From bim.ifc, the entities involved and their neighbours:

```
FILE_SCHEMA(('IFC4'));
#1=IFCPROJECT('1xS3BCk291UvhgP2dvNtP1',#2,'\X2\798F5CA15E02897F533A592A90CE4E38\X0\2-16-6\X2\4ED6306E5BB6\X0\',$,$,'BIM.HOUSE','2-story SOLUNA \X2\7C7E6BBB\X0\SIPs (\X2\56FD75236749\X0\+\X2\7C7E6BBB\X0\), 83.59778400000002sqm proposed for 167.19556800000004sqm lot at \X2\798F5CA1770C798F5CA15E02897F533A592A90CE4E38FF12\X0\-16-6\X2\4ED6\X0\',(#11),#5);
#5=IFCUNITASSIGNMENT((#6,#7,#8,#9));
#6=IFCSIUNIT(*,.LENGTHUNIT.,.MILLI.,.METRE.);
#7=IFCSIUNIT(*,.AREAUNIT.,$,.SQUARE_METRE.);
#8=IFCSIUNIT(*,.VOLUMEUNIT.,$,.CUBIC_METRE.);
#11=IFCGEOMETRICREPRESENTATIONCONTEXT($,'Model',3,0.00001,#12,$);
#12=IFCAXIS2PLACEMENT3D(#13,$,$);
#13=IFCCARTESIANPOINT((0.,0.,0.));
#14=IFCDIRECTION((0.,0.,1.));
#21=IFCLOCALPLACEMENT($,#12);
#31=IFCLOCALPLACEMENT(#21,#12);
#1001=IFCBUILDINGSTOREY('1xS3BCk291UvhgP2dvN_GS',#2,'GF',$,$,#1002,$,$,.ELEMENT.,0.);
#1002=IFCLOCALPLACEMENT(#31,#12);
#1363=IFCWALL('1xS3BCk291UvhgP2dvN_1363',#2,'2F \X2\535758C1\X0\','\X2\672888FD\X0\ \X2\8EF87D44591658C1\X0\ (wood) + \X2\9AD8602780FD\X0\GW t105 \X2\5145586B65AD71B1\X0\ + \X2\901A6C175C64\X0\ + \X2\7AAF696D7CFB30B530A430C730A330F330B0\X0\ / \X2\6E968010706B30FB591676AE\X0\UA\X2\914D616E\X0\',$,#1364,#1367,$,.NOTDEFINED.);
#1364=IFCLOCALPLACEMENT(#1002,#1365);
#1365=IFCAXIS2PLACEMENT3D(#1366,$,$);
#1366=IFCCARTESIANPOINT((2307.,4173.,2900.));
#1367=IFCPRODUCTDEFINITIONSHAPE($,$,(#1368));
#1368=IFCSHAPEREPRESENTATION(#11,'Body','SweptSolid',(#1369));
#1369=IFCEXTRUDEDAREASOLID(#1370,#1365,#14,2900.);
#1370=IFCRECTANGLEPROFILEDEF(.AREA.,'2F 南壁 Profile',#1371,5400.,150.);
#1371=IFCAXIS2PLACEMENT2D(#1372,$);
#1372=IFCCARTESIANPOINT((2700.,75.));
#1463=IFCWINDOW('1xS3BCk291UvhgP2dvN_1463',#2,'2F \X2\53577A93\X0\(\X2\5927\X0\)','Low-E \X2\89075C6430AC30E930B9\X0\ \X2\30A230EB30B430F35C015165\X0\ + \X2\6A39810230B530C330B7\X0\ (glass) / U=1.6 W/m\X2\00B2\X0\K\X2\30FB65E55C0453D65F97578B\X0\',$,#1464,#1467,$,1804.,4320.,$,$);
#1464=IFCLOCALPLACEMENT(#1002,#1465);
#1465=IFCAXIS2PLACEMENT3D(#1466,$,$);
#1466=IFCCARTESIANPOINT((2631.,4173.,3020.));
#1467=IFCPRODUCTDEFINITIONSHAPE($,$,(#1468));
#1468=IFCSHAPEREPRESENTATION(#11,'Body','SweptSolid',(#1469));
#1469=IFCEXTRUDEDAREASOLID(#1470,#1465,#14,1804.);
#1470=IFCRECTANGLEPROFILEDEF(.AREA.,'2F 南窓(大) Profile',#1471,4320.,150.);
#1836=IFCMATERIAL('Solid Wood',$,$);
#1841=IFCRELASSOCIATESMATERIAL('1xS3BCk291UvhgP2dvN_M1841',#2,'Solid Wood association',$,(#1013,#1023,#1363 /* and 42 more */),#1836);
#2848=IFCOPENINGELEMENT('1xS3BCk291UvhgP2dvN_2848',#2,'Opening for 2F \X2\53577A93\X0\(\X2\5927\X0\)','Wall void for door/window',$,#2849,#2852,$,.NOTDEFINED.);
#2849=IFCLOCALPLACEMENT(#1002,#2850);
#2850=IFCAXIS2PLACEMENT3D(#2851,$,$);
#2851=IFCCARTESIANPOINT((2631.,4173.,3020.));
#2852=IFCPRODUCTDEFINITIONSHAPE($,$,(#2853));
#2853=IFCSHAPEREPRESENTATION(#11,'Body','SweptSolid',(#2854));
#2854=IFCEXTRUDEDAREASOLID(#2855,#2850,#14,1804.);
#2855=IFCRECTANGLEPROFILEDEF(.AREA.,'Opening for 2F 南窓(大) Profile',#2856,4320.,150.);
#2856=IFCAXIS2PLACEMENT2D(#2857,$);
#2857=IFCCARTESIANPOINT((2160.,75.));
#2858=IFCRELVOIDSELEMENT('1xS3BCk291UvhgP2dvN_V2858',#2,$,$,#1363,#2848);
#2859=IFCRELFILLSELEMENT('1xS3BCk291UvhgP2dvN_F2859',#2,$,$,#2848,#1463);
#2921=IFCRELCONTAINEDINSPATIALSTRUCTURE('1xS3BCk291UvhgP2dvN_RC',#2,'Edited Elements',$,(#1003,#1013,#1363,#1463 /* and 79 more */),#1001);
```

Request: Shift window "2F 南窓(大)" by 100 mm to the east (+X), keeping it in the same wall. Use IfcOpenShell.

```python
import ifcopenshell
import ifcopenshell.api.geometry
import ifcopenshell.util.placement
import ifcopenshell.util.unit

model = ifcopenshell.open("bim.ifc")
unit_scale = ifcopenshell.util.unit.calculate_unit_scale(model)

window = model.by_guid("1xS3BCk291UvhgP2dvN_1463")
opening = window.FillsVoids[0].RelatingOpeningElement
wall = opening.VoidsElements[0].RelatingBuildingElement

wall_matrix = ifcopenshell.util.placement.get_local_placement(wall.ObjectPlacement)
shift = wall_matrix[:3, 0] * 0.1 / unit_scale
before = ifcopenshell.util.placement.get_local_placement(window.ObjectPlacement)[:3, 3].copy()

# The window is not placed relative to its opening, so move both.
for product in (opening, window):
    matrix = ifcopenshell.util.placement.get_local_placement(product.ObjectPlacement)
    matrix[:3, 3] += shift
    ifcopenshell.api.geometry.edit_object_placement(model, product=product, matrix=matrix, is_si=False)

after = ifcopenshell.util.placement.get_local_placement(window.ObjectPlacement)[:3, 3]
print("window moved by", (after - before).round(3) + 0.0)

model.write("bim-out.ifc")
```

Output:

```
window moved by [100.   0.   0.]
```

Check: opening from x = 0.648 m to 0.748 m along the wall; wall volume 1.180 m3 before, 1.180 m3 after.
